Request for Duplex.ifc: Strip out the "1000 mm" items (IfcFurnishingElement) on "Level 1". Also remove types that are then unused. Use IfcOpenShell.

First a look at what the model holds.

```python
import ifcopenshell
import ifcopenshell.util.element

model = ifcopenshell.open("Duplex.ifc")
print(model.schema)
storey = next(s for s in model.by_type("IfcBuildingStorey") if s.Name == "Level 1")
furniture = [e for e in ifcopenshell.util.element.get_decomposition(storey) if e.is_a("IfcFurnishingElement")]
seen = {}
for e in furniture:
    element_type = ifcopenshell.util.element.get_type(e)
    name = element_type.Name if element_type not in (None, e) else None
    seen[name] = seen.get(name, 0) + 1
for name, count in sorted(seen.items(), key=str):
    print(count, "x", name)
```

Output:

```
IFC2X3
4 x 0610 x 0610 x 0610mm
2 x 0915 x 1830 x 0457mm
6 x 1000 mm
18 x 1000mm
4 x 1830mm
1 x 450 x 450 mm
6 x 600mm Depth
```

```python
import ifcopenshell
import ifcopenshell.api.root
import ifcopenshell.util.element

model = ifcopenshell.open("Duplex.ifc")

storey = next(s for s in model.by_type("IfcBuildingStorey") if s.Name == "Level 1")
furniture = [e for e in ifcopenshell.util.element.get_decomposition(storey) if e.is_a("IfcFurnishingElement")]
targets = [e for e in furniture if (t := ifcopenshell.util.element.get_type(e)) not in (None, e) and t.Name == "1000 mm"]
types = {ifcopenshell.util.element.get_type(e) for e in targets} - {None, *targets}

for e in targets:
    ifcopenshell.api.root.remove_product(model, product=e)
print(len(targets), "removed")

unused = [t for t in types if not ifcopenshell.util.element.get_types(t)]
for t in unused:
    ifcopenshell.api.root.remove_product(model, product=t)
print(len(unused), "unused types removed")

model.write("Duplex_updated.ifc")
```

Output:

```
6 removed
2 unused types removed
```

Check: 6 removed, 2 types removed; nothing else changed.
